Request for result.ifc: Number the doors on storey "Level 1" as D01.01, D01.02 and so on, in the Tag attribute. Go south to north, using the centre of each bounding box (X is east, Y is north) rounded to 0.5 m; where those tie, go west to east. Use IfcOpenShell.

First a look at what the model holds.

```python
import ifcopenshell
import ifcopenshell.util.element
import ifcopenshell.util.placement

model = ifcopenshell.open("result.ifc")
print(model.schema)
storey = next(s for s in model.by_type("IfcBuildingStorey") if s.Name == "Level 1")
doors = [e for e in ifcopenshell.util.element.get_decomposition(storey) if e.is_a("IfcDoor")]
for e in sorted(doors, key=lambda e: e.id()):
    origin = ifcopenshell.util.placement.get_local_placement(e.ObjectPlacement)[:3, 3]
    print(e.id(), e.Tag, e.Name, origin.round(2) + 0.0, sep=" | ")
```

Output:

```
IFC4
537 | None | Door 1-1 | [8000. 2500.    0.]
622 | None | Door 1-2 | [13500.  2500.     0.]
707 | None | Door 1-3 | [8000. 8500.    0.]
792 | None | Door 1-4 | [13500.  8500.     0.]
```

```python
import ifcopenshell
import ifcopenshell.geom
import ifcopenshell.util.element
import ifcopenshell.util.shape

model = ifcopenshell.open("result.ifc")
settings = ifcopenshell.geom.settings()
settings.set("use-world-coords", True)


def centre(element):
    shape = ifcopenshell.geom.create_shape(settings, element)
    return ifcopenshell.util.shape.get_bbox_centroid(shape.geometry)


storey = next(s for s in model.by_type("IfcBuildingStorey") if s.Name == "Level 1")
doors = [e for e in ifcopenshell.util.element.get_decomposition(storey) if e.is_a("IfcDoor")]

# Insertion points can sit at a corner or the storey origin, so sort by the geometry (in metres).
centres = {e: centre(e) for e in doors}
doors.sort(key=lambda e: (round(centres[e][1] / 0.5), centres[e][0]))

for i, e in enumerate(doors, start=1):
    number = f"D01.{i:02d}"
    e.Tag = number
    print(e.id(), number)

model.write("result_updated.ifc")
```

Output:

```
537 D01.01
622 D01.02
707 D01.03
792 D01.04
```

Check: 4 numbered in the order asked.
